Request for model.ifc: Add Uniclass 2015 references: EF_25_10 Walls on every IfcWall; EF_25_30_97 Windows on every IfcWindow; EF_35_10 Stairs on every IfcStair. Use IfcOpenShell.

First a look at what the model holds.

```python
import ifcopenshell

model = ifcopenshell.open("model.ifc")
print(model.schema)
print("classifications:", [c.Name for c in model.by_type("IfcClassification")])
for ifc_class in ("IfcDoor", "IfcRoof", "IfcStair", "IfcWall", "IfcWindow"):
    print(ifc_class, len(model.by_type(ifc_class)))
```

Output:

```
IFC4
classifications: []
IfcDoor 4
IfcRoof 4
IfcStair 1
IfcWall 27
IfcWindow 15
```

```python
import ifcopenshell
import ifcopenshell.api.classification

model = ifcopenshell.open("model.ifc")

system = ifcopenshell.api.classification.add_classification(model, classification="Uniclass 2015")

codes = {
    "IfcWall": ("EF_25_10", "Walls"),
    "IfcWindow": ("EF_25_30_97", "Windows"),
    "IfcStair": ("EF_35_10", "Stairs"),
}
for ifc_class, (code, name) in codes.items():
    products = model.by_type(ifc_class)
    ifcopenshell.api.classification.add_reference(
        model, products=products, classification=system, identification=code, name=name
    )
    print(code, len(products))

model.write("model-out.ifc")
```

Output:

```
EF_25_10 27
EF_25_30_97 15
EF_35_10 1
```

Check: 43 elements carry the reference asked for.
